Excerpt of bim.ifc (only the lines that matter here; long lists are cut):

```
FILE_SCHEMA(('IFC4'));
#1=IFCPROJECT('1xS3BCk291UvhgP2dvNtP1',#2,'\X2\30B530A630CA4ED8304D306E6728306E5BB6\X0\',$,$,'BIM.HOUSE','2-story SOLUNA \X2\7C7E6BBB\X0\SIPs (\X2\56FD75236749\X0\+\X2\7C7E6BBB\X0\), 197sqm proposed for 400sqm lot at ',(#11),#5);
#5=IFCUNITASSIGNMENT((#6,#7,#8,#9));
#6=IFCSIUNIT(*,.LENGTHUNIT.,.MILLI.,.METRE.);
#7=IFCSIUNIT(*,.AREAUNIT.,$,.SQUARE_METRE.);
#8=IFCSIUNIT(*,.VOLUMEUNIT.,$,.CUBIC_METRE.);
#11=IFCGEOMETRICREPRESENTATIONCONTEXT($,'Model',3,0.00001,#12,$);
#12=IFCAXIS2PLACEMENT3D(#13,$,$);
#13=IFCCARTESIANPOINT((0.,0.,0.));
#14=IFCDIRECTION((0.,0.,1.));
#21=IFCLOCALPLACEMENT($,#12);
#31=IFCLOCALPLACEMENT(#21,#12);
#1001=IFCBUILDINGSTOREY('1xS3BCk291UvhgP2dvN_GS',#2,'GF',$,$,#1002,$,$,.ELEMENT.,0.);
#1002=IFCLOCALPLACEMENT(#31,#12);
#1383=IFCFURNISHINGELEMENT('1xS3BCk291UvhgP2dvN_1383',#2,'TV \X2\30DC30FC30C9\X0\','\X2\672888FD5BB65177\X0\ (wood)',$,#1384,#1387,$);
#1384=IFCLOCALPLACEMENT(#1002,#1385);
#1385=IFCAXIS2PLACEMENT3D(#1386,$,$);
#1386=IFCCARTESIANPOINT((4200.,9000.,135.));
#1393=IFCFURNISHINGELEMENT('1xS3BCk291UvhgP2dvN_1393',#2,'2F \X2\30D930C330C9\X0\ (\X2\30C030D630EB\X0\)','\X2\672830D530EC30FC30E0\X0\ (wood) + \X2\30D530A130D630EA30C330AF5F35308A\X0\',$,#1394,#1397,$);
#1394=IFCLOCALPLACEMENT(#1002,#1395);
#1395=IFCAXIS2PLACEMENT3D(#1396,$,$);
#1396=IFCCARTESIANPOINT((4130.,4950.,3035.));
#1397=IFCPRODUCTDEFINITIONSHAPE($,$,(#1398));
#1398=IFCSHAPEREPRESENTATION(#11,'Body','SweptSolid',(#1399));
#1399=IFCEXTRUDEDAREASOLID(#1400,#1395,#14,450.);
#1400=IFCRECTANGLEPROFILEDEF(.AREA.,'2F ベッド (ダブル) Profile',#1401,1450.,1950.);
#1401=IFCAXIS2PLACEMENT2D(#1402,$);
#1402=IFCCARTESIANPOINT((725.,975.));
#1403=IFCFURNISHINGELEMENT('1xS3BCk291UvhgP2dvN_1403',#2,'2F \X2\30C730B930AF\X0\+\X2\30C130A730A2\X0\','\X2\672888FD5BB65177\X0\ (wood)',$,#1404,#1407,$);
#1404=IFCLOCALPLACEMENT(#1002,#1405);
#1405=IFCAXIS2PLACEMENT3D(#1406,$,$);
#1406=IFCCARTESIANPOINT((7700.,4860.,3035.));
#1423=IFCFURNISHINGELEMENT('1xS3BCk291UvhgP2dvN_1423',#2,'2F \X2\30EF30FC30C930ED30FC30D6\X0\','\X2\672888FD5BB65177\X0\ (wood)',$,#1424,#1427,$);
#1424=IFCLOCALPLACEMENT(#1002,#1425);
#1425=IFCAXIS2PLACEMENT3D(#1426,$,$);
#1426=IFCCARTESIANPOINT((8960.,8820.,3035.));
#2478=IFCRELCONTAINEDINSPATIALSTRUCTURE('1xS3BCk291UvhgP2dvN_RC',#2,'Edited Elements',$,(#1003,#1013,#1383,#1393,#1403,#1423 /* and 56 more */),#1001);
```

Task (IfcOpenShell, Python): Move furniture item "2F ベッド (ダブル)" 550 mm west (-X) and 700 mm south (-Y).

```python
import ifcopenshell
import ifcopenshell.api.geometry
import ifcopenshell.util.placement
import ifcopenshell.util.unit

model = ifcopenshell.open("bim.ifc")
unit_scale = ifcopenshell.util.unit.calculate_unit_scale(model)

item = model.by_id(1393)
matrix = ifcopenshell.util.placement.get_local_placement(item.ObjectPlacement)
matrix[0, 3] -= 0.55 / unit_scale
matrix[1, 3] -= 0.7 / unit_scale
ifcopenshell.api.geometry.edit_object_placement(model, product=item, matrix=matrix, is_si=False)

print(ifcopenshell.util.placement.get_local_placement(item.ObjectPlacement).round(3) + 0.0)

model.write("bim-out.ifc")
```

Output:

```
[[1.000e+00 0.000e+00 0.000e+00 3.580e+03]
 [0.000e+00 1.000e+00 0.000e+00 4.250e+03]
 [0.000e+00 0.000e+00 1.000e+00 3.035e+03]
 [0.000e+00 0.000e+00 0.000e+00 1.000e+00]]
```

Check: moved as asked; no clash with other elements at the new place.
